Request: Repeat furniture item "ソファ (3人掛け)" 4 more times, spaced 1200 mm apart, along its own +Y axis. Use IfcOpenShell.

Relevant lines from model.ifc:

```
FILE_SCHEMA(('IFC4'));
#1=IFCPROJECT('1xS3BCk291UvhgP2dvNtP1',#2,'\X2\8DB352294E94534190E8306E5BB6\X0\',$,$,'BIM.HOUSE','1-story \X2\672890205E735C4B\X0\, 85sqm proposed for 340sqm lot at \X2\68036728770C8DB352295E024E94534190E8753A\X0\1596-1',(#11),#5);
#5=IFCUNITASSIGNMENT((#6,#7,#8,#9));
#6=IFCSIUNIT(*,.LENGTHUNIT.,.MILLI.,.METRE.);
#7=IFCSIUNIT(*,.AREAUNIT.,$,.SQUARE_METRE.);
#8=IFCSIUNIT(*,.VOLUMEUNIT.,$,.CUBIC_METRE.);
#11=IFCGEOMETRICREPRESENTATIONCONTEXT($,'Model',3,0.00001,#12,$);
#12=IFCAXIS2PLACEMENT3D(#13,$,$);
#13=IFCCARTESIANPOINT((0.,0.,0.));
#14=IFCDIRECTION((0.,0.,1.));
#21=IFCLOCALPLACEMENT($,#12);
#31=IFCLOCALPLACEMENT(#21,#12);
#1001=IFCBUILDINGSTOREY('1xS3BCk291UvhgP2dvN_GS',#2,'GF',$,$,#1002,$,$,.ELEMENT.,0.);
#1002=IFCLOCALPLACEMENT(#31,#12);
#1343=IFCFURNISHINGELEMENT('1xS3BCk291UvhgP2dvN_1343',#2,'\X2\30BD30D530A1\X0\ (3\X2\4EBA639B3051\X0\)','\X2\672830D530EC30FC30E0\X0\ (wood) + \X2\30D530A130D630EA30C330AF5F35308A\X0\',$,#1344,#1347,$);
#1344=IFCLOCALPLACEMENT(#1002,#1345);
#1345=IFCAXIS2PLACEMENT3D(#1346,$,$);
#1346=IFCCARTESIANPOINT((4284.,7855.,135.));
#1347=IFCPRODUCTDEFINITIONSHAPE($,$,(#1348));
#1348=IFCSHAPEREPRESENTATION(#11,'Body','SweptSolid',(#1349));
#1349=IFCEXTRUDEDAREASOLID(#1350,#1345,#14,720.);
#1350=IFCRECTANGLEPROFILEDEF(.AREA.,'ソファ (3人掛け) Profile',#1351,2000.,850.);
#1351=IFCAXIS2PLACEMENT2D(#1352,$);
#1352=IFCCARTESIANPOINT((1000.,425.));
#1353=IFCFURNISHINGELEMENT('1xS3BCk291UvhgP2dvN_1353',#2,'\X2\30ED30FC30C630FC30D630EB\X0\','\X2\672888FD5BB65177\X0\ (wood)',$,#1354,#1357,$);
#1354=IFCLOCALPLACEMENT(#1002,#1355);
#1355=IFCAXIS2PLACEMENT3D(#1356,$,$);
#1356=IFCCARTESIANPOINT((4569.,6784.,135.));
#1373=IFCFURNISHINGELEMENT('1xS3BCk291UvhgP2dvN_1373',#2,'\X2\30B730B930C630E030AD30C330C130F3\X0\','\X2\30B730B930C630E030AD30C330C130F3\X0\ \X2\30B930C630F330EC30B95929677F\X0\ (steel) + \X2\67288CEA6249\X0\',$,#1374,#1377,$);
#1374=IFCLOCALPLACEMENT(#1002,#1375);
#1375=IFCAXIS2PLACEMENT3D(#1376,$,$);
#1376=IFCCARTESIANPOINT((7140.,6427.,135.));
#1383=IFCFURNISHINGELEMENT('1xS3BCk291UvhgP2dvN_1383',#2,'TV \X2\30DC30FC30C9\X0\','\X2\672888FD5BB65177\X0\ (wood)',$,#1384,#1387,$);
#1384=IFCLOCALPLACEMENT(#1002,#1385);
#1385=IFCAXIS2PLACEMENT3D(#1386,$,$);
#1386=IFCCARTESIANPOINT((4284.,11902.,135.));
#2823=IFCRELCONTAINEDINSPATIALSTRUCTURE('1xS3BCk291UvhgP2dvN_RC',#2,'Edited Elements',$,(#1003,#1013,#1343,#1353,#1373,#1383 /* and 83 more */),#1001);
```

```python
import ifcopenshell
import ifcopenshell.api.geometry
import ifcopenshell.api.root
import ifcopenshell.util.element
import ifcopenshell.util.placement
import ifcopenshell.util.unit

model = ifcopenshell.open("model.ifc")
unit_scale = ifcopenshell.util.unit.calculate_unit_scale(model)


def reuse_history(source, copy):
    """copy_class also copies each property set's owner history, people and application; keep the originals."""
    for rel in copy.IsDefinedBy:
        if rel.is_a("IfcRelDefinesByProperties") and (history := rel.RelatingPropertyDefinition.OwnerHistory):
            rel.RelatingPropertyDefinition.OwnerHistory = source.OwnerHistory
            ifcopenshell.util.element.remove_deep2(model, history)


source = model.by_guid("1xS3BCk291UvhgP2dvN_1343")
base = ifcopenshell.util.placement.get_local_placement(source.ObjectPlacement)
step = base[:3, 1] * 1.2 / unit_scale

for i in range(1, 5):
    copy = ifcopenshell.api.root.copy_class(model, product=source)
    copy.Representation = ifcopenshell.util.element.copy_deep(
        model, source.Representation, exclude=["IfcGeometricRepresentationContext", "IfcRepresentationMap"]
    )
    reuse_history(source, copy)
    matrix = base.copy()
    matrix[:3, 3] += i * step
    print("added at", matrix[:3, 3].round(3) + 0.0)
    ifcopenshell.api.geometry.edit_object_placement(model, product=copy, matrix=matrix, is_si=False)

model.write("model_updated.ifc")
```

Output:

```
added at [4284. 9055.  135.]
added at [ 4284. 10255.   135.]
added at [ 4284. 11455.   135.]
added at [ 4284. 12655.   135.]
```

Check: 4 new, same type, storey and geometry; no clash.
